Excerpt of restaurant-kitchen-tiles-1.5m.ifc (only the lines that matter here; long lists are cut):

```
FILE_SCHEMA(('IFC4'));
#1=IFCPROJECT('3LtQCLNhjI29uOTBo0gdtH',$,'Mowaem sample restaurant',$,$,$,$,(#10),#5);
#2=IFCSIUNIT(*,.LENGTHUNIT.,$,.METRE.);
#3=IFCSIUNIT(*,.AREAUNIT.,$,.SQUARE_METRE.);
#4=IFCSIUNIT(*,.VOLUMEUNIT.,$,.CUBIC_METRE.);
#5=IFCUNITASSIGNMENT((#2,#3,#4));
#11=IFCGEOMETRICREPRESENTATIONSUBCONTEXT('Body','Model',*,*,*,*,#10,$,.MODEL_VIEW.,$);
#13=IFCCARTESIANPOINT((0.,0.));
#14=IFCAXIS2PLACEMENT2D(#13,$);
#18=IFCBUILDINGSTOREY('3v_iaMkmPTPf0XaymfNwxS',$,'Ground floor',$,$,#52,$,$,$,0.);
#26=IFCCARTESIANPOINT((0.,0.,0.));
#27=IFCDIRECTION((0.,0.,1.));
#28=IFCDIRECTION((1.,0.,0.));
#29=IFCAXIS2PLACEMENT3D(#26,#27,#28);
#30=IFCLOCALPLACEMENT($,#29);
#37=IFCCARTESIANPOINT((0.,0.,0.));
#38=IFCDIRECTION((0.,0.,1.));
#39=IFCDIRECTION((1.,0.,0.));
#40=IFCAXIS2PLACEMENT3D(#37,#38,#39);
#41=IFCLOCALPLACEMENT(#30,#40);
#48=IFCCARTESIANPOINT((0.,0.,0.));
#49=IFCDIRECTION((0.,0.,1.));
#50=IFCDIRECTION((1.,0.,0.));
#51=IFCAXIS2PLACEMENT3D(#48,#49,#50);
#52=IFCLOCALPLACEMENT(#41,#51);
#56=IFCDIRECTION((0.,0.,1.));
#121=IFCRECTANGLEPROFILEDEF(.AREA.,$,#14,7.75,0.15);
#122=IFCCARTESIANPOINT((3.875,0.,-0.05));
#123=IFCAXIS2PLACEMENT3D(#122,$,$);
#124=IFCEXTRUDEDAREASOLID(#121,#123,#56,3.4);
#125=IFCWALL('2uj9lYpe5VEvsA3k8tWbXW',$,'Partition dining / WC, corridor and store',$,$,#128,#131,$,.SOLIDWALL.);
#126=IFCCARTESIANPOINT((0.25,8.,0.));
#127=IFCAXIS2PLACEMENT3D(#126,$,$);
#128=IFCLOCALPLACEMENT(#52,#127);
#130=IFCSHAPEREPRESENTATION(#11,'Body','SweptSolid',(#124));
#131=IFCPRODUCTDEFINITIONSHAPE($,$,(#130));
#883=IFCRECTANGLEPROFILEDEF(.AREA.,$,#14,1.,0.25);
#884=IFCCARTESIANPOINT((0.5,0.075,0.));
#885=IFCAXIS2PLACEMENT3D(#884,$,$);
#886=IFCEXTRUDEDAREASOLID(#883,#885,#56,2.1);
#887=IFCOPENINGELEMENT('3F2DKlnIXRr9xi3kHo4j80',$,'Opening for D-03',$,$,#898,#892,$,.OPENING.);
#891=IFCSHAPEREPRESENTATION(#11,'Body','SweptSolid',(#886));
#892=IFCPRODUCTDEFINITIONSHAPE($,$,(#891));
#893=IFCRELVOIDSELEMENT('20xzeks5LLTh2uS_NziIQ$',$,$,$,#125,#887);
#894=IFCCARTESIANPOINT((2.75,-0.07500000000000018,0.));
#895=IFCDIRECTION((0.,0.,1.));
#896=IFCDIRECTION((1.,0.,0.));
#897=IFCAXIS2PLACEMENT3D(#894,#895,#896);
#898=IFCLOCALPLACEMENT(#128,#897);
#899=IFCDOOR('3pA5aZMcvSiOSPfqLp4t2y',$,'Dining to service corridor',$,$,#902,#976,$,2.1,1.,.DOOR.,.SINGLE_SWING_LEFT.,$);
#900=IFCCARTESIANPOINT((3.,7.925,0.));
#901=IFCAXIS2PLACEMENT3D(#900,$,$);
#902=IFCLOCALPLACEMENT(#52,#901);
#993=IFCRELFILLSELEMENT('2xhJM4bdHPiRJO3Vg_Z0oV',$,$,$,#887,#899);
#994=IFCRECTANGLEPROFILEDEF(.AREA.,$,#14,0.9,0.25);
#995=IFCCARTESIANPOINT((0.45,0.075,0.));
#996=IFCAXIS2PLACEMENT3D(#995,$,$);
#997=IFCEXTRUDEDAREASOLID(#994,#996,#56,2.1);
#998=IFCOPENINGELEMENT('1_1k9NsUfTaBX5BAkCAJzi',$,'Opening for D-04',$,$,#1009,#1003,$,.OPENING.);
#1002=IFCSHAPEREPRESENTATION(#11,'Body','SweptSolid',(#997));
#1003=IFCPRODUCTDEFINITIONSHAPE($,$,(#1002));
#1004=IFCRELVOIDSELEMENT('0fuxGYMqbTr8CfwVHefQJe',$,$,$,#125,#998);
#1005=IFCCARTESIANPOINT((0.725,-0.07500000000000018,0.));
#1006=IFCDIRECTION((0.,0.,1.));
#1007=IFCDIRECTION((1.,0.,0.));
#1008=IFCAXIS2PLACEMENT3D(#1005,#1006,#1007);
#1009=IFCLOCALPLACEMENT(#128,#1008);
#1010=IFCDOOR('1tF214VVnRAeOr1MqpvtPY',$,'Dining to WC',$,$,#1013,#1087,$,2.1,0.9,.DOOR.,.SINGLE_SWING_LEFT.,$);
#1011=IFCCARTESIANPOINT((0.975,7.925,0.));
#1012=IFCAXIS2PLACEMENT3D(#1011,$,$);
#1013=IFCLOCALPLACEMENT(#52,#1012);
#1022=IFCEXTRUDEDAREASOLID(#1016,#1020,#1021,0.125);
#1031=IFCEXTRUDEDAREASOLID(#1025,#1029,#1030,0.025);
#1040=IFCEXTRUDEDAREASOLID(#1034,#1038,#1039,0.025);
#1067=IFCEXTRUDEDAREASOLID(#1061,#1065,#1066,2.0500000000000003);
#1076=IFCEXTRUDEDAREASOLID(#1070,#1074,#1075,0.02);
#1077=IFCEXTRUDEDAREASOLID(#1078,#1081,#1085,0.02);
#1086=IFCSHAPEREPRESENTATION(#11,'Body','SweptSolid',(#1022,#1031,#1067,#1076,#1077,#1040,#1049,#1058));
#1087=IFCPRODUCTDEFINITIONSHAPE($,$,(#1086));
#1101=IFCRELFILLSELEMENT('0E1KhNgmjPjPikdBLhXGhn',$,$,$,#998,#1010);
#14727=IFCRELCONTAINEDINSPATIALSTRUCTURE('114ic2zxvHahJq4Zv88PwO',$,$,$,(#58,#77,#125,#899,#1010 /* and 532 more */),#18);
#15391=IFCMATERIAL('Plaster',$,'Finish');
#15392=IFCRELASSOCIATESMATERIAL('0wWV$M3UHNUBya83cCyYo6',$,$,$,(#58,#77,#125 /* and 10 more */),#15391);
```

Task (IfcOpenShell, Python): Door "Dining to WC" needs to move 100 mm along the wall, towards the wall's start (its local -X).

```python
import ifcopenshell
import ifcopenshell.api.geometry
import ifcopenshell.util.placement
import ifcopenshell.util.unit

model = ifcopenshell.open("restaurant-kitchen-tiles-1.5m.ifc")
unit_scale = ifcopenshell.util.unit.calculate_unit_scale(model)

door = model.by_guid("1tF214VVnRAeOr1MqpvtPY")
opening = door.FillsVoids[0].RelatingOpeningElement
wall = opening.VoidsElements[0].RelatingBuildingElement

wall_matrix = ifcopenshell.util.placement.get_local_placement(wall.ObjectPlacement)
shift = wall_matrix[:3, 0] * -0.1 / unit_scale
before = ifcopenshell.util.placement.get_local_placement(door.ObjectPlacement)[:3, 3].copy()

# The door is not placed relative to its opening, so move both.
for product in (opening, door):
    matrix = ifcopenshell.util.placement.get_local_placement(product.ObjectPlacement)
    matrix[:3, 3] += shift
    ifcopenshell.api.geometry.edit_object_placement(model, product=product, matrix=matrix, is_si=False)

after = ifcopenshell.util.placement.get_local_placement(door.ObjectPlacement)[:3, 3]
print("door moved by", (after - before).round(3) + 0.0)

model.write("restaurant-kitchen-tiles-1.5m_rev.ifc")
```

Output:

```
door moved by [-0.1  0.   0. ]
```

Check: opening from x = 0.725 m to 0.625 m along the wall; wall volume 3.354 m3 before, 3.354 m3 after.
